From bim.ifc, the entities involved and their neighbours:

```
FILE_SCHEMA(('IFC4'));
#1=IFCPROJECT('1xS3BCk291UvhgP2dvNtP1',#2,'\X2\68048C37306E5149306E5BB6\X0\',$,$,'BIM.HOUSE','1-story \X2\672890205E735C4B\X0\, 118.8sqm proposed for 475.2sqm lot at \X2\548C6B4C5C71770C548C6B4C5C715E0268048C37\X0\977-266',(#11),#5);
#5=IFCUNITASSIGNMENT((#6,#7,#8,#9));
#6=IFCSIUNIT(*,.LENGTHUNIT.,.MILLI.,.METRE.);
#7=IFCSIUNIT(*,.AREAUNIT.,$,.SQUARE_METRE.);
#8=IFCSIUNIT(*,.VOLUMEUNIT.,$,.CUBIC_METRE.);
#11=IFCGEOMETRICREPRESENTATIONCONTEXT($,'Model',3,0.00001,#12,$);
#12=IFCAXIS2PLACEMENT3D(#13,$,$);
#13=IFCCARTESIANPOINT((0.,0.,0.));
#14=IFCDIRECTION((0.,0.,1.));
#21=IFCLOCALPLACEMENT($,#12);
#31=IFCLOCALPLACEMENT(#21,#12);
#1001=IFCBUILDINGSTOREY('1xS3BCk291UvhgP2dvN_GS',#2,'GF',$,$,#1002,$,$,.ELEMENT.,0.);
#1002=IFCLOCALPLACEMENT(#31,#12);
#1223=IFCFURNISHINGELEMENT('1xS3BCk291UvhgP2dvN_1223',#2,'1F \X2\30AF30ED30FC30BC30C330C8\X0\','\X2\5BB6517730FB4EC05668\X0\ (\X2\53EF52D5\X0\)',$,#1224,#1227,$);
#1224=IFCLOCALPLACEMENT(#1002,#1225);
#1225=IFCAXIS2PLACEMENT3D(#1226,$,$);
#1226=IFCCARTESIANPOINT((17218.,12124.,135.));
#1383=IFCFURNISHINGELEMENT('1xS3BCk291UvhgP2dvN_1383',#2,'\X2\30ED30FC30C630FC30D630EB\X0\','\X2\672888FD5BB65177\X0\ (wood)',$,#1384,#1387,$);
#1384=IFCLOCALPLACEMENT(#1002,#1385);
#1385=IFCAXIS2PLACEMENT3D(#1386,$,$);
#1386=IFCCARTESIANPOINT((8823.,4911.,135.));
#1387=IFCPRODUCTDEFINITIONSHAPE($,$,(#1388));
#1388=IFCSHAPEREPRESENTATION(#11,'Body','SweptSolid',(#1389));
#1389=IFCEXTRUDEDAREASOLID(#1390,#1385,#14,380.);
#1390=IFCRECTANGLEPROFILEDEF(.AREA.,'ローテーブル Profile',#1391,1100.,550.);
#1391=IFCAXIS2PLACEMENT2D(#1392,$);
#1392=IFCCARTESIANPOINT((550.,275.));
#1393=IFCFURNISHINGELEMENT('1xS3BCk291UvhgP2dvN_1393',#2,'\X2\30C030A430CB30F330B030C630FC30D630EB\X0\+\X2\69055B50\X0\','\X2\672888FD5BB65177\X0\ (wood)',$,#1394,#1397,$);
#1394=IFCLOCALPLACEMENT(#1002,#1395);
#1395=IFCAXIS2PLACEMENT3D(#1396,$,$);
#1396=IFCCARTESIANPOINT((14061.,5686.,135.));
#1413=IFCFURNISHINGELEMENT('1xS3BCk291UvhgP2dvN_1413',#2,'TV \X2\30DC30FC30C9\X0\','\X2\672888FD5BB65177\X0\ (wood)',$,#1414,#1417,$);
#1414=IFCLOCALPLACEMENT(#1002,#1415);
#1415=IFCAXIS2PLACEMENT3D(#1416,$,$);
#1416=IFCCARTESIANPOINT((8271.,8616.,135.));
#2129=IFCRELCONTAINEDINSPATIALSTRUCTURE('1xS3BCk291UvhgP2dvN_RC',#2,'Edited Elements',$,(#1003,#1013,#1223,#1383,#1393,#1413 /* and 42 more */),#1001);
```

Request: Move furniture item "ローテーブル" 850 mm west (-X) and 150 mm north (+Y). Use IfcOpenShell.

```python
import ifcopenshell
import ifcopenshell.api.geometry
import ifcopenshell.util.placement

model = ifcopenshell.open("bim.ifc")

item = model.by_id(1383)
matrix = ifcopenshell.util.placement.get_local_placement(item.ObjectPlacement)
matrix[0, 3] -= 850.0
matrix[1, 3] += 150.0
ifcopenshell.api.geometry.edit_object_placement(model, product=item, matrix=matrix, is_si=False)

print(ifcopenshell.util.placement.get_local_placement(item.ObjectPlacement).round(3) + 0.0)

model.write("bim_edited.ifc")
```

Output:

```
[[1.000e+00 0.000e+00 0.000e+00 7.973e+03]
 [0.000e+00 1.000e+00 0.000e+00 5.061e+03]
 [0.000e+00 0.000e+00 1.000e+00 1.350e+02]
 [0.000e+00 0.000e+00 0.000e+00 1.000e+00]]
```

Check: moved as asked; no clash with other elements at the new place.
